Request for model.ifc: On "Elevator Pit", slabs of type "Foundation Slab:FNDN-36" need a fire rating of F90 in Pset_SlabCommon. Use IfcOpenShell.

First a look at what the model holds.

```python
import ifcopenshell
import ifcopenshell.util.element

model = ifcopenshell.open("model.ifc")
print(model.schema)
storey = next(s for s in model.by_type("IfcBuildingStorey") if s.Name == "Elevator Pit")
slabs = [e for e in ifcopenshell.util.element.get_decomposition(storey) if e.is_a("IfcSlab")]
seen = {}
for e in slabs:
    element_type = ifcopenshell.util.element.get_type(e)
    key = (element_type.Name if element_type != e and element_type else None, ifcopenshell.util.element.get_pset(e, "Pset_SlabCommon", "FireRating"))
    seen[key] = seen.get(key, 0) + 1
for (name, value), count in sorted(seen.items(), key=str):
    print(count, "x", name, "|", value)
```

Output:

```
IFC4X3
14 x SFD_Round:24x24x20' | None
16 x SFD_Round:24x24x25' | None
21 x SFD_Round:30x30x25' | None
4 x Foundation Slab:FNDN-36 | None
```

```python
import ifcopenshell
import ifcopenshell.api.pset
import ifcopenshell.util.element

model = ifcopenshell.open("model.ifc")

storey = next(s for s in model.by_type("IfcBuildingStorey") if s.Name == "Elevator Pit")
slabs = [e for e in ifcopenshell.util.element.get_decomposition(storey) if e.is_a("IfcSlab")]

count = 0
for e in slabs:
    element_type = ifcopenshell.util.element.get_type(e)
    if element_type in (None, e) or element_type.Name != "Foundation Slab:FNDN-36":
        continue
    # add_pset returns the element's existing set when there is one.
    pset = ifcopenshell.api.pset.add_pset(model, product=e, name="Pset_SlabCommon")
    ifcopenshell.api.pset.edit_pset(model, pset=pset, properties={"FireRating": "F90"})
    count += 1

print(count, "slabs updated")

model.write("model_updated.ifc")
```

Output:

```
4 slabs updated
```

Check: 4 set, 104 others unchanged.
